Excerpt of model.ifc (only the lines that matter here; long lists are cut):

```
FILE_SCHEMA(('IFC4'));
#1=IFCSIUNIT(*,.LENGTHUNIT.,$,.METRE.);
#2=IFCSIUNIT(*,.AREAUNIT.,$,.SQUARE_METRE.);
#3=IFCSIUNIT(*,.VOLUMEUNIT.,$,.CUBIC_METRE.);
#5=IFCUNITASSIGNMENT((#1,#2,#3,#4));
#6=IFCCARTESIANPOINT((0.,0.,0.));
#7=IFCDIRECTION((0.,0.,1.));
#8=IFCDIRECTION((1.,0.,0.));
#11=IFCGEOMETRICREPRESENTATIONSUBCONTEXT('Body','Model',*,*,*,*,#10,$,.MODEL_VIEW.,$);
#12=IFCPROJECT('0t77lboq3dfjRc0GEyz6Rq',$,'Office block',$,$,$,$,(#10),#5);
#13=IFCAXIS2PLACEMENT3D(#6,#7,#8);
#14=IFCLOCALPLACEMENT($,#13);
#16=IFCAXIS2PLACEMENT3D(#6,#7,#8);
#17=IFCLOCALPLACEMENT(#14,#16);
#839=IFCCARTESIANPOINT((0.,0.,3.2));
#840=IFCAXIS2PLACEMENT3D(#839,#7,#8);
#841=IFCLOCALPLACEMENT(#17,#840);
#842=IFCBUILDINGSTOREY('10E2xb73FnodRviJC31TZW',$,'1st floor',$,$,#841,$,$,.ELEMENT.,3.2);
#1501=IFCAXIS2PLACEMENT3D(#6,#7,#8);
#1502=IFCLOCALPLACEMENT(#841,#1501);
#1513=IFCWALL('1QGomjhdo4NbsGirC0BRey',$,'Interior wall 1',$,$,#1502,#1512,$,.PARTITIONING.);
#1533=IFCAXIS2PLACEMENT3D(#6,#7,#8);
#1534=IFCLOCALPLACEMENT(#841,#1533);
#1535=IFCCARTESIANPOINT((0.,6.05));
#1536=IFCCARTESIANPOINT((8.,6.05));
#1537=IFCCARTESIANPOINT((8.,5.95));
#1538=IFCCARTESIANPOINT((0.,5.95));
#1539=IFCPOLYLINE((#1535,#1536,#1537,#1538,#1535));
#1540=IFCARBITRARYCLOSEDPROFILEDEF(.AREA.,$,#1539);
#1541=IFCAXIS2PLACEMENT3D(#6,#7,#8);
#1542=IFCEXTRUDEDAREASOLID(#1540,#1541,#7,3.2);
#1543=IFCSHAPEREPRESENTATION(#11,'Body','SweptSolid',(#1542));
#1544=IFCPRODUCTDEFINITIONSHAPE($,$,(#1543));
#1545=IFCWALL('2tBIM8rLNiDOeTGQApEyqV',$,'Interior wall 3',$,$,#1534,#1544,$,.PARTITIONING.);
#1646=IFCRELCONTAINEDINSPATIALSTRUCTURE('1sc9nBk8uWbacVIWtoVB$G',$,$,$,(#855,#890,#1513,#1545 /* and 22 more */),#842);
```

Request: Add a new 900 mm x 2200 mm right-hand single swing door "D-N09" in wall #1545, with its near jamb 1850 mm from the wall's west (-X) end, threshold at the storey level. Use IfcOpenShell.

```python
import numpy as np
import ifcopenshell
import ifcopenshell.api.feature
import ifcopenshell.api.geometry
import ifcopenshell.api.root
import ifcopenshell.api.spatial
import ifcopenshell.geom
import ifcopenshell.util.element
import ifcopenshell.util.placement
import ifcopenshell.util.representation
import ifcopenshell.util.shape
import ifcopenshell.util.unit

model = ifcopenshell.open("model.ifc")
unit_scale = ifcopenshell.util.unit.calculate_unit_scale(model)
settings = ifcopenshell.geom.settings()


def volume(element):
    """Net volume in cubic metres, openings subtracted."""
    shape = ifcopenshell.geom.create_shape(settings, element)
    return ifcopenshell.util.shape.get_volume(shape.geometry)


wall = model.by_guid("2tBIM8rLNiDOeTGQApEyqV")
storey = ifcopenshell.util.element.get_container(wall, ifc_class="IfcBuildingStorey")
context = ifcopenshell.util.representation.get_context(model, "Model", "Body", "MODEL_VIEW")
before = volume(wall)

width, height, from_end, sill = 0.9, 2.2, 1.85, 0.0  # metres

# The wall runs along its own X axis, and the end named is its -X end.
wall_shape = ifcopenshell.geom.create_shape(settings, wall)
x, y, z = ifcopenshell.util.shape.get_vertices(wall_shape.geometry).T
start = x.min() + from_end
face, thickness = float(y.min()), float(y.max() - y.min())
wall_matrix = ifcopenshell.util.placement.get_local_placement(wall.ObjectPlacement)
level = ifcopenshell.util.placement.get_local_placement(storey.ObjectPlacement)[2, 3]


def in_wall(x, y):
    """Placement at x, y metres in the wall's axes, at sill height."""
    matrix = wall_matrix.copy()
    matrix[:, 3] = wall_matrix @ np.array([x / unit_scale, y / unit_scale, 0.0, 1.0])
    matrix[2, 3] = level + sill / unit_scale
    return matrix


# Opening: a box that overshoots both wall faces by 50 mm.
opening = ifcopenshell.api.root.create_entity(model, ifc_class="IfcOpeningElement", predefined_type="OPENING")
box = ifcopenshell.api.geometry.add_wall_representation(
    model, context=context, length=width, height=height, thickness=thickness + 0.1
)
ifcopenshell.api.geometry.assign_representation(model, product=opening, representation=box)
ifcopenshell.api.geometry.edit_object_placement(model, product=opening, matrix=in_wall(start, face - 0.05), is_si=False)
ifcopenshell.api.feature.add_feature(model, feature=opening, element=wall)

door = ifcopenshell.api.root.create_entity(model, ifc_class="IfcDoor", name="D-N09", predefined_type="DOOR")
door.OverallWidth, door.OverallHeight = width / unit_scale, height / unit_scale
door.OperationType = "SINGLE_SWING_RIGHT"
body = ifcopenshell.api.geometry.add_door_representation(
    model,
    context=context,
    overall_width=door.OverallWidth,
    overall_height=door.OverallHeight,
    operation_type="SINGLE_SWING_RIGHT",
    lining_properties={"LiningDepth": thickness / unit_scale, "ThresholdDepth": thickness / unit_scale},
)
ifcopenshell.api.geometry.assign_representation(model, product=door, representation=body)
ifcopenshell.api.spatial.assign_container(model, products=[door], relating_structure=storey)
ifcopenshell.api.feature.add_filling(model, opening=opening, element=door)

# The lining spans the wall, so the door starts at the wall face.
ifcopenshell.api.geometry.edit_object_placement(model, product=door, matrix=in_wall(start, face), is_si=False)

after = volume(wall)

print(f"wall volume {before:.3f} -> {after:.3f} m3")

model.write("model-out.ifc")
```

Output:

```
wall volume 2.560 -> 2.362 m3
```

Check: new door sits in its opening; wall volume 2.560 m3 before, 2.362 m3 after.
